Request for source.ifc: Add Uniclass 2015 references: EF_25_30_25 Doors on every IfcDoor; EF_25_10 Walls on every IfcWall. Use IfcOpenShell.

First a look at what the model holds.

```python
import ifcopenshell

model = ifcopenshell.open("source.ifc")
print(model.schema)
print("classifications:", [c.Name for c in model.by_type("IfcClassification")])
for ifc_class in ("IfcDoor", "IfcRoof", "IfcStair", "IfcWall", "IfcWindow"):
    print(ifc_class, len(model.by_type(ifc_class)))
```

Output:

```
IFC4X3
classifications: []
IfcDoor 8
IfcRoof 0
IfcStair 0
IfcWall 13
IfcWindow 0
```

```python
import ifcopenshell
import ifcopenshell.api.classification

model = ifcopenshell.open("source.ifc")

system = ifcopenshell.api.classification.add_classification(model, classification="Uniclass 2015")

codes = {
    "IfcDoor": ("EF_25_30_25", "Doors"),
    "IfcWall": ("EF_25_10", "Walls"),
}
for ifc_class, (code, name) in codes.items():
    products = model.by_type(ifc_class)
    ifcopenshell.api.classification.add_reference(
        model, products=products, classification=system, identification=code, name=name
    )
    print(code, len(products))

model.write("source_updated.ifc")
```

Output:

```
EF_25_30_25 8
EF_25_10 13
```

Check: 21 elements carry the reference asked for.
